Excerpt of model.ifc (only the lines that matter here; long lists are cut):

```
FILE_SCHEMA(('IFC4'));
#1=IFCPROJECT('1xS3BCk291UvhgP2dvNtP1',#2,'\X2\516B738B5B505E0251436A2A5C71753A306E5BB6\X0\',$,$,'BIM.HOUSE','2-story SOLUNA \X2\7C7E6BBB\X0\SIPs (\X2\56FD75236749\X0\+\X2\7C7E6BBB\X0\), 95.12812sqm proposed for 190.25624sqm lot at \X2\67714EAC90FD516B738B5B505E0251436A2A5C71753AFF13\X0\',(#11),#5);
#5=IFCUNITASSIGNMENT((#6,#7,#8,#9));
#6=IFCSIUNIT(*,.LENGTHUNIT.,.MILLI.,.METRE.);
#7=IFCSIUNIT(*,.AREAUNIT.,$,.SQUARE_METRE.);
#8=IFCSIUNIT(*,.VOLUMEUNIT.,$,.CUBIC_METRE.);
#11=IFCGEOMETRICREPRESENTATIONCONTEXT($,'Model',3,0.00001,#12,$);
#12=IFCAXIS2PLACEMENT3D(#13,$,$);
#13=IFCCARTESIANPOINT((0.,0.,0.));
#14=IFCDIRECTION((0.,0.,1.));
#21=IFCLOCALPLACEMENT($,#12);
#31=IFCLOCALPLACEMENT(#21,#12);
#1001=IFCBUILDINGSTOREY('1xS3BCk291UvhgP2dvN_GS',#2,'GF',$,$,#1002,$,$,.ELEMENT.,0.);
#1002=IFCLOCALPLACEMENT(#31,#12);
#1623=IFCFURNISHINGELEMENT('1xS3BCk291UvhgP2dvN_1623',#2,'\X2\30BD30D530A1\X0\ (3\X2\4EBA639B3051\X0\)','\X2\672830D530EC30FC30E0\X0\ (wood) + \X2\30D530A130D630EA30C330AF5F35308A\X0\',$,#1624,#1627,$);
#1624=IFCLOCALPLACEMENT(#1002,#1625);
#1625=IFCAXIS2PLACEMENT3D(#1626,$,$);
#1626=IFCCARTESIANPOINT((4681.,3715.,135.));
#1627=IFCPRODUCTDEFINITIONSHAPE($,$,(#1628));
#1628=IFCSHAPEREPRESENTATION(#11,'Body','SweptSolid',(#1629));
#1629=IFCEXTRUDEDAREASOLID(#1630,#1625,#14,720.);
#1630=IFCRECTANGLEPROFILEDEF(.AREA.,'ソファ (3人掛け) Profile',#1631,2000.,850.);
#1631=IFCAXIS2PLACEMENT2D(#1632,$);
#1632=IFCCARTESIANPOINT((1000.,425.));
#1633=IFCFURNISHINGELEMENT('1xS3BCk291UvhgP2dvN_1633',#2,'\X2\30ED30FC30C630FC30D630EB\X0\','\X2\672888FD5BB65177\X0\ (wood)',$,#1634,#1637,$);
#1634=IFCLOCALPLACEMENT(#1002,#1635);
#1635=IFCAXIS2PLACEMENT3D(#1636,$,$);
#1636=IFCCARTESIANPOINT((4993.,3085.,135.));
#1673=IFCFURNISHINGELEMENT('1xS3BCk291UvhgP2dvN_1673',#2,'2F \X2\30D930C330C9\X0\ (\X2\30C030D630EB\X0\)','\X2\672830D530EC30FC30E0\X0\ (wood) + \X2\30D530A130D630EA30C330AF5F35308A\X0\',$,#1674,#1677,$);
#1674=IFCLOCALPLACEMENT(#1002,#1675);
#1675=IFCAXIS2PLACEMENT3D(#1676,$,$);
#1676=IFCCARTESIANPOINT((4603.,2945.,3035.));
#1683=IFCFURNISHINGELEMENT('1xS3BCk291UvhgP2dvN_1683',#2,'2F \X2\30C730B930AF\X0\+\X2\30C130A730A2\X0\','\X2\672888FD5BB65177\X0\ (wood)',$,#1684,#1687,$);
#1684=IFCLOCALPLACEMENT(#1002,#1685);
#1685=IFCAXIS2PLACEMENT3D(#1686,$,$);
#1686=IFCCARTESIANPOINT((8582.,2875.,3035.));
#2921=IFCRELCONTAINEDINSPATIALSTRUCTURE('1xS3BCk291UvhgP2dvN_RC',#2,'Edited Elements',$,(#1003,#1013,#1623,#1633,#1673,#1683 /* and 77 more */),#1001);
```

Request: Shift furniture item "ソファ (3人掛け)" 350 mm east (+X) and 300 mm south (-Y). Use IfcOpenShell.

```python
import ifcopenshell
import ifcopenshell.api.geometry
import ifcopenshell.util.placement

model = ifcopenshell.open("model.ifc")

item = model.by_guid("1xS3BCk291UvhgP2dvN_1623")
matrix = ifcopenshell.util.placement.get_local_placement(item.ObjectPlacement)
matrix[0, 3] += 350.0
matrix[1, 3] -= 300.0
ifcopenshell.api.geometry.edit_object_placement(model, product=item, matrix=matrix, is_si=False)

print(ifcopenshell.util.placement.get_local_placement(item.ObjectPlacement).round(3) + 0.0)

model.write("model-out.ifc")
```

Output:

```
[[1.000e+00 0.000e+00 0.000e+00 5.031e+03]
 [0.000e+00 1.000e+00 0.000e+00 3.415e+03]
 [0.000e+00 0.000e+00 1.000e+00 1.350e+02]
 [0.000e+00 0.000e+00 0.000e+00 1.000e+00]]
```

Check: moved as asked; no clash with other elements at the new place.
